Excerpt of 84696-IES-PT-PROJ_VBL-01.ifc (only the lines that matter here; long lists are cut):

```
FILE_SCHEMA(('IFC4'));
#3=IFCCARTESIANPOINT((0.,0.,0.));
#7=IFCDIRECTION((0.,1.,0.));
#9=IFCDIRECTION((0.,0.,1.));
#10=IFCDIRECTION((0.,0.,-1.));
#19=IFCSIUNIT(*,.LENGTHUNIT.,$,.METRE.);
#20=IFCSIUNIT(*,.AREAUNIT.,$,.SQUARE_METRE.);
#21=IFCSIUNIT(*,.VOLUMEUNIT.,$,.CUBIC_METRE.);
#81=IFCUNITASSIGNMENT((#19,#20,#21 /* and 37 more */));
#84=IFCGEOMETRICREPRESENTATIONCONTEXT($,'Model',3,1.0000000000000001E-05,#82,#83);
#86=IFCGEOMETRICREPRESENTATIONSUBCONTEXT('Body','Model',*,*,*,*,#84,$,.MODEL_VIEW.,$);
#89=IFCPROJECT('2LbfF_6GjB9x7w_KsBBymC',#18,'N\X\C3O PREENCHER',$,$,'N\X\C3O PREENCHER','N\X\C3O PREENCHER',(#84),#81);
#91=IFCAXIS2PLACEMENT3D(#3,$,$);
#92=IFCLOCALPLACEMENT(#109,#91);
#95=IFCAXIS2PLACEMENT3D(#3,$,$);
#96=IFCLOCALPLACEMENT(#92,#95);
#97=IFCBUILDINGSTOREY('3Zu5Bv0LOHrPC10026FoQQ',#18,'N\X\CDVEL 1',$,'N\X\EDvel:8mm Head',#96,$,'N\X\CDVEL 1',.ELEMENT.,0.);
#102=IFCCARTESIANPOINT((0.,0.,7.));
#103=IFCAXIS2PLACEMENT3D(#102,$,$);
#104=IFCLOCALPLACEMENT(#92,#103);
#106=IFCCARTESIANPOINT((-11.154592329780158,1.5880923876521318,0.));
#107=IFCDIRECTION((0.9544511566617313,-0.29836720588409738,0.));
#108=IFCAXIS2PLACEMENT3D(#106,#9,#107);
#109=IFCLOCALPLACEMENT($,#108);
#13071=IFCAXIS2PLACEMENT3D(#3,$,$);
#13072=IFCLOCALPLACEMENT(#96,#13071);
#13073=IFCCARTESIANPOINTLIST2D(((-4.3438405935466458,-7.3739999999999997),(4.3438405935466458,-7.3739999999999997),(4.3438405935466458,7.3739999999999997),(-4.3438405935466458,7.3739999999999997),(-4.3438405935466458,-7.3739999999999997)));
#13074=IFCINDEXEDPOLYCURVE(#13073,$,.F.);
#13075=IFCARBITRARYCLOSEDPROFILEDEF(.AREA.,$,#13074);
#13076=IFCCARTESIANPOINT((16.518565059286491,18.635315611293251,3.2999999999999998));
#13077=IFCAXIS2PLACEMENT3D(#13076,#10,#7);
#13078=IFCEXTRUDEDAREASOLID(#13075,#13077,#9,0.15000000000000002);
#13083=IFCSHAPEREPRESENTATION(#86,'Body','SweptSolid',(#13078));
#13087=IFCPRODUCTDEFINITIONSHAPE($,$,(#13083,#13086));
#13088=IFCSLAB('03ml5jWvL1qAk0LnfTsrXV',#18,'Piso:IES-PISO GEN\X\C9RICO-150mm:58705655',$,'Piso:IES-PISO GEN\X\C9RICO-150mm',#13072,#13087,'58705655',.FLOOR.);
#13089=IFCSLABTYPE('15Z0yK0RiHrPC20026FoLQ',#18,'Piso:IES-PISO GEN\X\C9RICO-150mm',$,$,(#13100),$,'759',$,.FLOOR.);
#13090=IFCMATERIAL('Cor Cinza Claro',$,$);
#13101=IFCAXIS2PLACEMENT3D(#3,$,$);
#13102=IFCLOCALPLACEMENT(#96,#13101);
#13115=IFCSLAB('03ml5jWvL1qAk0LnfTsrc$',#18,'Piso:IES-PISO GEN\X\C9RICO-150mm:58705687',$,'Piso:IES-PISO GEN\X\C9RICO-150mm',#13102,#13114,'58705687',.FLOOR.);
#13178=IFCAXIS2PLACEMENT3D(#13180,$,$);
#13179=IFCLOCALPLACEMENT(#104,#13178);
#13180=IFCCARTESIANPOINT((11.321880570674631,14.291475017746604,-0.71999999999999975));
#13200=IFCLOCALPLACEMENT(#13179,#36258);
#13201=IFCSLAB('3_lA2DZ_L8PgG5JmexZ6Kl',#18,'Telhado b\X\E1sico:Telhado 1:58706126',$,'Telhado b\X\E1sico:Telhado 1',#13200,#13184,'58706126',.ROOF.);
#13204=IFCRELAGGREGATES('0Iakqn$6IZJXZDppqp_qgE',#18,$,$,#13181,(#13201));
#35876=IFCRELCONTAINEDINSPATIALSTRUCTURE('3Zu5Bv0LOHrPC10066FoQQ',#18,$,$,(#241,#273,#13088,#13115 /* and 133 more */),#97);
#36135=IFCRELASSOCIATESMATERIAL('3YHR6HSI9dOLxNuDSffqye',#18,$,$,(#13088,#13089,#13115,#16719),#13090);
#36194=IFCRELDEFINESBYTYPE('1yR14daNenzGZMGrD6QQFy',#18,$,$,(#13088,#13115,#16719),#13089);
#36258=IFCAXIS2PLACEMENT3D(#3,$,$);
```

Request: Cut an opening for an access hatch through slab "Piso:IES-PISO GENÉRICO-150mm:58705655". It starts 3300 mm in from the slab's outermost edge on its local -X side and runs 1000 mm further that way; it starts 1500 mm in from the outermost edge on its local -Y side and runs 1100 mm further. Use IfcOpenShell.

```python
import numpy as np
import ifcopenshell
import ifcopenshell.api.feature
import ifcopenshell.api.geometry
import ifcopenshell.api.root
import ifcopenshell.geom
import ifcopenshell.util.placement
import ifcopenshell.util.representation
import ifcopenshell.util.shape
import ifcopenshell.util.unit

model = ifcopenshell.open("84696-IES-PT-PROJ_VBL-01.ifc")
unit_scale = ifcopenshell.util.unit.calculate_unit_scale(model)
settings = ifcopenshell.geom.settings()


def volume(element):
    """Net volume in cubic metres, openings subtracted."""
    shape = ifcopenshell.geom.create_shape(settings, element)
    return ifcopenshell.util.shape.get_volume(shape.geometry)


slab = model.by_guid("03ml5jWvL1qAk0LnfTsrXV")
before = volume(slab)

# Extent in the slab's own axes, in metres. The edges named are its -X and -Y sides.
slab_shape = ifcopenshell.geom.create_shape(settings, slab)
vertices = ifcopenshell.util.shape.get_vertices(slab_shape.geometry)
x_min, y_min, bottom = vertices.min(axis=0)
top = vertices[:, 2].max()

opening = ifcopenshell.api.root.create_entity(model, ifc_class="IfcOpeningElement", name="Access hatch opening", predefined_type="OPENING")
context = ifcopenshell.util.representation.get_context(model, "Model", "Body", "MODEL_VIEW")
width, depth = 1, 1.1
outline = [(0.0, 0.0), (width, 0.0), (width, depth), (0.0, depth), (0.0, 0.0)]
# Overshoot both faces by 50 mm so the cut is clean.
shape = ifcopenshell.api.geometry.add_slab_representation(
    model, context=context, depth=top - bottom + 0.1, polyline=outline
)
ifcopenshell.api.geometry.assign_representation(model, product=opening, representation=shape)

matrix = ifcopenshell.util.placement.get_local_placement(slab.ObjectPlacement)
matrix[:, 3] = matrix @ np.append(np.array([x_min + 3.3, y_min + 1.5, bottom - 0.05]) / unit_scale, 1.0)
ifcopenshell.api.geometry.edit_object_placement(model, product=opening, matrix=matrix, is_si=False)
ifcopenshell.api.feature.add_feature(model, feature=opening, element=slab)

after = volume(slab)

print(f"slab volume {before:.3f} -> {after:.3f} m3")

model.write("84696-IES-PT-PROJ_VBL-01_updated.ifc")
```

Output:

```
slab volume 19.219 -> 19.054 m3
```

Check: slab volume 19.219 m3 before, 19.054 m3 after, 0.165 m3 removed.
